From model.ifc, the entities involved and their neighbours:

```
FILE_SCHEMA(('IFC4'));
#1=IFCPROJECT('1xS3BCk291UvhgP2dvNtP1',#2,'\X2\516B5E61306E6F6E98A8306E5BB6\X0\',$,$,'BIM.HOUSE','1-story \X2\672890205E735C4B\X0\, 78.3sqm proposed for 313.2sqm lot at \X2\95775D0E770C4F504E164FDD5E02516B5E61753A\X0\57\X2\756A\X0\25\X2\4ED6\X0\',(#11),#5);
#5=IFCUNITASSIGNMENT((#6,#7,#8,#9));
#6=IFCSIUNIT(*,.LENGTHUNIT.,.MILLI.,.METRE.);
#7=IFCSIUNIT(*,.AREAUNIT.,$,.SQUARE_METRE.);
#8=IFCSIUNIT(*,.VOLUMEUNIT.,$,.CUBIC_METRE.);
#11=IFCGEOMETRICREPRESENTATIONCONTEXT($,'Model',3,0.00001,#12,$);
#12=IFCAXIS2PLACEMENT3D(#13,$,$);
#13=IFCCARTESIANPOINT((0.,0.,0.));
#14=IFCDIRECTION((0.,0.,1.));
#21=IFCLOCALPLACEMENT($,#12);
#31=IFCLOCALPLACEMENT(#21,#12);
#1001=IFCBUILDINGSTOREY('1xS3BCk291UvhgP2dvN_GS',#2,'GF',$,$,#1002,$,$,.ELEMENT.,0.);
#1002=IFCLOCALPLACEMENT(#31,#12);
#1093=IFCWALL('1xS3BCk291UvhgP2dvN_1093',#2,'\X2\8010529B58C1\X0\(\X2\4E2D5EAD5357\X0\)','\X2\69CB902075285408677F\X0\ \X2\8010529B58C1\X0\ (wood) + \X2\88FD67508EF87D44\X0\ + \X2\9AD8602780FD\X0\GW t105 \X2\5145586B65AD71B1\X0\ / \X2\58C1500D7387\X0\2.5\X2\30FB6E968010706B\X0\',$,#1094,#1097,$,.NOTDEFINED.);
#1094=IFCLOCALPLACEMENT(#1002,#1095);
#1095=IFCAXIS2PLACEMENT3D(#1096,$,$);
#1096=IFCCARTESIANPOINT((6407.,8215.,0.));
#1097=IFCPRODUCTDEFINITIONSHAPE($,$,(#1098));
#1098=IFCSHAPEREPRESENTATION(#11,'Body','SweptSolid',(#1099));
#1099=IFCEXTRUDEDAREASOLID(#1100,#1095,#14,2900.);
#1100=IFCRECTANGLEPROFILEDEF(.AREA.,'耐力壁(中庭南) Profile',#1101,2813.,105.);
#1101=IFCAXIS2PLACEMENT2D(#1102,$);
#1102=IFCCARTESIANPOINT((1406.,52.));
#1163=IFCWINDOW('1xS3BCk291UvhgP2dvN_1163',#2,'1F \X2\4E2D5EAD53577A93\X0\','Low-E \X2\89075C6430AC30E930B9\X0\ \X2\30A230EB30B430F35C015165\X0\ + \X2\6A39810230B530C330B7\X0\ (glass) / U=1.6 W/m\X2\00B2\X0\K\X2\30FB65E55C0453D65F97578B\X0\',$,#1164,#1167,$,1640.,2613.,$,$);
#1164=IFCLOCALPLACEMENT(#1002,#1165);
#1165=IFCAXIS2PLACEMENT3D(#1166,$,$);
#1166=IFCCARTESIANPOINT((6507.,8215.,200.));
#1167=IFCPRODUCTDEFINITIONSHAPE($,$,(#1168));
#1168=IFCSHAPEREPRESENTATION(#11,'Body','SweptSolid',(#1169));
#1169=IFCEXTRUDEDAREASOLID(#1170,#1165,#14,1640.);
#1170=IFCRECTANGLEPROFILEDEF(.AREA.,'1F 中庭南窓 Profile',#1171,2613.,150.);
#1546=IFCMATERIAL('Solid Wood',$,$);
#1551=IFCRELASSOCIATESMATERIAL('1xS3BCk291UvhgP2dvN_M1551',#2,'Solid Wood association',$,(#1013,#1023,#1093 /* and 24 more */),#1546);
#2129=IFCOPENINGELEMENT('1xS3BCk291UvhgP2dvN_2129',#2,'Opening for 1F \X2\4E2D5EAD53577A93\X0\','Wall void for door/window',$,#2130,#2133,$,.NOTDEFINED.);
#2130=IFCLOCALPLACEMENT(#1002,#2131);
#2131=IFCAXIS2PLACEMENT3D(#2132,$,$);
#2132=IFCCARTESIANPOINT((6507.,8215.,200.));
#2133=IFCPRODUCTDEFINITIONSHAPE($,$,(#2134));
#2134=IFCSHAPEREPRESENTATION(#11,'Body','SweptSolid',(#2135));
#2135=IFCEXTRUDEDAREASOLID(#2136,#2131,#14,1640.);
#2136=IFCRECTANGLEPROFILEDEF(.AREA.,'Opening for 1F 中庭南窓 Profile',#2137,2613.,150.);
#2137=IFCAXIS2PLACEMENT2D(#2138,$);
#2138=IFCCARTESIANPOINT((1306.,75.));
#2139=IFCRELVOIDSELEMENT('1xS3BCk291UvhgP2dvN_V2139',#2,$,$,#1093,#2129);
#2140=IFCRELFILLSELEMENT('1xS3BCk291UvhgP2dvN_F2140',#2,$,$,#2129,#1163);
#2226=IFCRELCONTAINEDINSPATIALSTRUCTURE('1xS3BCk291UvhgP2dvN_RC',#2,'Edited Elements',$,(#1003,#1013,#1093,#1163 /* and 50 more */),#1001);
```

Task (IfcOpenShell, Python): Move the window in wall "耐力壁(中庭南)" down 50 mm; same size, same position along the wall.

```python
import numpy as np
import ifcopenshell
import ifcopenshell.api.geometry
import ifcopenshell.util.placement
import ifcopenshell.util.unit

model = ifcopenshell.open("model.ifc")
unit_scale = ifcopenshell.util.unit.calculate_unit_scale(model)

window = model.by_guid("1xS3BCk291UvhgP2dvN_1163")
opening = window.FillsVoids[0].RelatingOpeningElement
dz = -0.05 / unit_scale

shift = np.array([0.0, 0.0, dz])
# The window is not placed relative to its opening, so move both.
for product in (opening, window):
    matrix = ifcopenshell.util.placement.get_local_placement(product.ObjectPlacement)
    matrix[:3, 3] += shift
    ifcopenshell.api.geometry.edit_object_placement(model, product=product, matrix=matrix, is_si=False)

print(f"moved by {dz * unit_scale:+.3f} m")

model.write("model_rev.ifc")
```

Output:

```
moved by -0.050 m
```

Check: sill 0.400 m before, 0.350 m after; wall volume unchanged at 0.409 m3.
